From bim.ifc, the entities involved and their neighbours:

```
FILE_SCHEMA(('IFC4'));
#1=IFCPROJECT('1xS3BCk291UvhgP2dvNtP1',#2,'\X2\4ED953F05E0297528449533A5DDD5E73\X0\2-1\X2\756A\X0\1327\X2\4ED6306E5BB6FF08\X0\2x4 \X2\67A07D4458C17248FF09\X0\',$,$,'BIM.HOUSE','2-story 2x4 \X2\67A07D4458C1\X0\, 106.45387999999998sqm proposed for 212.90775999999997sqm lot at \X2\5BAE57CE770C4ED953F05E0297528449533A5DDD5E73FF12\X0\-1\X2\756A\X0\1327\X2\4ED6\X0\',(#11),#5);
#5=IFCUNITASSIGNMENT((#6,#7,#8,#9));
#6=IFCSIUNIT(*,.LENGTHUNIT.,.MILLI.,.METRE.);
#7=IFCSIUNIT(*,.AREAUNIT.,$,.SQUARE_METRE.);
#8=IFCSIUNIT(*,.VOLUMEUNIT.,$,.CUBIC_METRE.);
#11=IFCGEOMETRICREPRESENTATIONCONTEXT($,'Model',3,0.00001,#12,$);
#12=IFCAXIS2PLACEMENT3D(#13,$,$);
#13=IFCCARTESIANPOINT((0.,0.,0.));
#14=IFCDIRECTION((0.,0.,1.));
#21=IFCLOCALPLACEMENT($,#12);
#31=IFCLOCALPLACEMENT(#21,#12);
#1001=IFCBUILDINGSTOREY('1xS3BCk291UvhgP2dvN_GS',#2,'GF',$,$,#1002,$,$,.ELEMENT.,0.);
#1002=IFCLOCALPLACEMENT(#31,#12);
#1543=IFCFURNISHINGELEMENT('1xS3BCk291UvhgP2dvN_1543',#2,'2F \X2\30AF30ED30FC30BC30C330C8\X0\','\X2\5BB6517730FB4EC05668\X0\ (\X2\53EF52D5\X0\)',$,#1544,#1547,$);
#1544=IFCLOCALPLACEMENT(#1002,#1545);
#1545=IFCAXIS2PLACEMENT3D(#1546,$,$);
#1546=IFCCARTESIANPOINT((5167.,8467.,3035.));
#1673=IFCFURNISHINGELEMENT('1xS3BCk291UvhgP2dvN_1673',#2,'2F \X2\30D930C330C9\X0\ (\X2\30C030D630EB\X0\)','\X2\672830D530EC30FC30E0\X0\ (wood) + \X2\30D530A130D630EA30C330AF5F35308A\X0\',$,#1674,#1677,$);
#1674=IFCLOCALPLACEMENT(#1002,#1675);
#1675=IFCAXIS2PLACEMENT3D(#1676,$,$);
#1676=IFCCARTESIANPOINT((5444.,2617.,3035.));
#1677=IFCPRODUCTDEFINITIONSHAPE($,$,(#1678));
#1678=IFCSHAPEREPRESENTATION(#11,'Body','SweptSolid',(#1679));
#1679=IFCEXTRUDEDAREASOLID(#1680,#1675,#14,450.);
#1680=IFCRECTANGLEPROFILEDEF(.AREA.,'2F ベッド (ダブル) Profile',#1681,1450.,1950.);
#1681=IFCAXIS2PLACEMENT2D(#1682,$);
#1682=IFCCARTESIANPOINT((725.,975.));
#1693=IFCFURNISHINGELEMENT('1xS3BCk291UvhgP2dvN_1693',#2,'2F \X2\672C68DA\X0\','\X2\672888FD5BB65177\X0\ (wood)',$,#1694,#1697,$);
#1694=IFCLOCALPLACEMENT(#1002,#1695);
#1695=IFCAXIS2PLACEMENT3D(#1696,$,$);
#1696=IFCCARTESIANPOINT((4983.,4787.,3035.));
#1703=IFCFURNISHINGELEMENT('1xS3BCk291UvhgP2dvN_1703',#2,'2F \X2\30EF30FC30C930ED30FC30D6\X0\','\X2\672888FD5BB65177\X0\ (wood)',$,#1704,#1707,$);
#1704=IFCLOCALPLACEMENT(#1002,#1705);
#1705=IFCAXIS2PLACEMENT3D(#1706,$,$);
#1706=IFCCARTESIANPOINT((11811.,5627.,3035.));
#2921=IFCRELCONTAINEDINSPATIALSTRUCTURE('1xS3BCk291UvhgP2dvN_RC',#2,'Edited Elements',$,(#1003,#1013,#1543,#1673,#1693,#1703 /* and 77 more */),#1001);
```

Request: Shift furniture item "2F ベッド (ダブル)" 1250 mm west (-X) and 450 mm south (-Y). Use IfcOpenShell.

```python
import ifcopenshell
import ifcopenshell.api.geometry
import ifcopenshell.util.placement
import ifcopenshell.util.unit

model = ifcopenshell.open("bim.ifc")
unit_scale = ifcopenshell.util.unit.calculate_unit_scale(model)

item = model.by_guid("1xS3BCk291UvhgP2dvN_1673")
matrix = ifcopenshell.util.placement.get_local_placement(item.ObjectPlacement)
matrix[0, 3] -= 1.25 / unit_scale
matrix[1, 3] -= 0.45 / unit_scale
ifcopenshell.api.geometry.edit_object_placement(model, product=item, matrix=matrix, is_si=False)

print(ifcopenshell.util.placement.get_local_placement(item.ObjectPlacement).round(3) + 0.0)

model.write("bim_edited.ifc")
```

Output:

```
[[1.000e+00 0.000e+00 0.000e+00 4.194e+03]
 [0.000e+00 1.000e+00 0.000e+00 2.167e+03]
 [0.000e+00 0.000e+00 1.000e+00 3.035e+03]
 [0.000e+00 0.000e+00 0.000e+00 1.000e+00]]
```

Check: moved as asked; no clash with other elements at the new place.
